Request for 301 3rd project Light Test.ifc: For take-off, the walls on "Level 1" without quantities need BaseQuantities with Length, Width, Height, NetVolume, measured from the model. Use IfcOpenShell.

First a look at what the model holds.

```python
import ifcopenshell
import ifcopenshell.util.element
import ifcopenshell.util.unit

model = ifcopenshell.open("301 3rd project Light Test.ifc")
print(model.schema)
for unit_type in ("LENGTHUNIT", "AREAUNIT", "VOLUMEUNIT"):
    print(unit_type, ifcopenshell.util.unit.calculate_unit_scale(model, unit_type))
storey = next(s for s in model.by_type("IfcBuildingStorey") if s.Name == "Level 1")
walls = [e for e in ifcopenshell.util.element.get_decomposition(storey) if e.is_a("IfcWall")]
for e in sorted(walls, key=lambda e: e.id()):
    print(e.id(), e.is_a(), e.Name, list(ifcopenshell.util.element.get_psets(e, qtos_only=True)), sep=" | ")
```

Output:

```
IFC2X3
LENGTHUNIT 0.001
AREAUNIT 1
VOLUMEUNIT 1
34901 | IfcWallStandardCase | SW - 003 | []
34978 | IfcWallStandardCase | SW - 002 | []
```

```python
import ifcopenshell
import ifcopenshell.api.pset
import ifcopenshell.geom
import ifcopenshell.util.element
import ifcopenshell.util.shape
import ifcopenshell.util.unit

model = ifcopenshell.open("301 3rd project Light Test.ifc")
unit_scale = ifcopenshell.util.unit.calculate_unit_scale(model)
volume_scale = ifcopenshell.util.unit.calculate_unit_scale(model, "VOLUMEUNIT")
settings = ifcopenshell.geom.settings()

storey = next(s for s in model.by_type("IfcBuildingStorey") if s.Name == "Level 1")
walls = [e for e in ifcopenshell.util.element.get_decomposition(storey) if e.is_a("IfcWall")]

for e in sorted(walls, key=lambda e: e.id()):
    if ifcopenshell.util.element.get_psets(e, qtos_only=True, should_inherit=False):
        continue
    # Geometry comes back in metres, in the element's own axes.
    shape = ifcopenshell.geom.create_shape(settings, e)
    values = {
        "Length": ifcopenshell.util.shape.get_x(shape.geometry) / unit_scale,
        "Width": ifcopenshell.util.shape.get_y(shape.geometry) / unit_scale,
        "Height": ifcopenshell.util.shape.get_z(shape.geometry) / unit_scale,
        "NetVolume": ifcopenshell.util.shape.get_volume(shape.geometry) / volume_scale,
    }
    qto = ifcopenshell.api.pset.add_qto(model, product=e, name="BaseQuantities")
    ifcopenshell.api.pset.edit_qto(model, qto=qto, properties=values)
    print(e.id(), {k: round(v, 3) for k, v in values.items()})

model.write("301 3rd project Light Test_v2.ifc")
```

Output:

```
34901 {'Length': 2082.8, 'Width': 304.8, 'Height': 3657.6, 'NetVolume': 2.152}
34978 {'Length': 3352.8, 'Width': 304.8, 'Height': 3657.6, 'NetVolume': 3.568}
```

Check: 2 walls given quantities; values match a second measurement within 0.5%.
